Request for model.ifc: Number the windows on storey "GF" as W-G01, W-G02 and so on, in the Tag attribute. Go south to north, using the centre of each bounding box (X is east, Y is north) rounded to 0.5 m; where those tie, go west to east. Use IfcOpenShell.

First a look at what the model holds.

```python
import ifcopenshell
import ifcopenshell.util.element
import ifcopenshell.util.placement

model = ifcopenshell.open("model.ifc")
print(model.schema)
storey = next(s for s in model.by_type("IfcBuildingStorey") if s.Name == "GF")
windows = [e for e in ifcopenshell.util.element.get_decomposition(storey) if e.is_a("IfcWindow")]
for e in sorted(windows, key=lambda e: e.id()):
    origin = ifcopenshell.util.placement.get_local_placement(e.ObjectPlacement)[:3, 3]
    print(e.id(), e.Tag, e.Name, origin.round(2) + 0.0, sep=" | ")
```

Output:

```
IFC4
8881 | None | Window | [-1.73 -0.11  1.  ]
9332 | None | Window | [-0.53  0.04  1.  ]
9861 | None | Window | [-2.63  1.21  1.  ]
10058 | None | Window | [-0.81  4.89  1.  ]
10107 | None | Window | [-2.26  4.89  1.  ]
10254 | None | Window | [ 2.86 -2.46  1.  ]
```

```python
import ifcopenshell
import ifcopenshell.geom
import ifcopenshell.util.element
import ifcopenshell.util.shape

model = ifcopenshell.open("model.ifc")
settings = ifcopenshell.geom.settings()
settings.set("use-world-coords", True)


def centre(element):
    shape = ifcopenshell.geom.create_shape(settings, element)
    return ifcopenshell.util.shape.get_bbox_centroid(shape.geometry)


storey = next(s for s in model.by_type("IfcBuildingStorey") if s.Name == "GF")
windows = [e for e in ifcopenshell.util.element.get_decomposition(storey) if e.is_a("IfcWindow")]

# Insertion points can sit at a corner or the storey origin, so sort by the geometry (in metres).
centres = {e: centre(e) for e in windows}
windows.sort(key=lambda e: (round(centres[e][1] / 0.5), centres[e][0]))

for i, e in enumerate(windows, start=1):
    number = f"W-G{i:02d}"
    e.Tag = number
    print(e.id(), number)

model.write("model-out.ifc")
```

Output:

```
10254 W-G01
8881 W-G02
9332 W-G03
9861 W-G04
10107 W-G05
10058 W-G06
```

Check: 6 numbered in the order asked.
